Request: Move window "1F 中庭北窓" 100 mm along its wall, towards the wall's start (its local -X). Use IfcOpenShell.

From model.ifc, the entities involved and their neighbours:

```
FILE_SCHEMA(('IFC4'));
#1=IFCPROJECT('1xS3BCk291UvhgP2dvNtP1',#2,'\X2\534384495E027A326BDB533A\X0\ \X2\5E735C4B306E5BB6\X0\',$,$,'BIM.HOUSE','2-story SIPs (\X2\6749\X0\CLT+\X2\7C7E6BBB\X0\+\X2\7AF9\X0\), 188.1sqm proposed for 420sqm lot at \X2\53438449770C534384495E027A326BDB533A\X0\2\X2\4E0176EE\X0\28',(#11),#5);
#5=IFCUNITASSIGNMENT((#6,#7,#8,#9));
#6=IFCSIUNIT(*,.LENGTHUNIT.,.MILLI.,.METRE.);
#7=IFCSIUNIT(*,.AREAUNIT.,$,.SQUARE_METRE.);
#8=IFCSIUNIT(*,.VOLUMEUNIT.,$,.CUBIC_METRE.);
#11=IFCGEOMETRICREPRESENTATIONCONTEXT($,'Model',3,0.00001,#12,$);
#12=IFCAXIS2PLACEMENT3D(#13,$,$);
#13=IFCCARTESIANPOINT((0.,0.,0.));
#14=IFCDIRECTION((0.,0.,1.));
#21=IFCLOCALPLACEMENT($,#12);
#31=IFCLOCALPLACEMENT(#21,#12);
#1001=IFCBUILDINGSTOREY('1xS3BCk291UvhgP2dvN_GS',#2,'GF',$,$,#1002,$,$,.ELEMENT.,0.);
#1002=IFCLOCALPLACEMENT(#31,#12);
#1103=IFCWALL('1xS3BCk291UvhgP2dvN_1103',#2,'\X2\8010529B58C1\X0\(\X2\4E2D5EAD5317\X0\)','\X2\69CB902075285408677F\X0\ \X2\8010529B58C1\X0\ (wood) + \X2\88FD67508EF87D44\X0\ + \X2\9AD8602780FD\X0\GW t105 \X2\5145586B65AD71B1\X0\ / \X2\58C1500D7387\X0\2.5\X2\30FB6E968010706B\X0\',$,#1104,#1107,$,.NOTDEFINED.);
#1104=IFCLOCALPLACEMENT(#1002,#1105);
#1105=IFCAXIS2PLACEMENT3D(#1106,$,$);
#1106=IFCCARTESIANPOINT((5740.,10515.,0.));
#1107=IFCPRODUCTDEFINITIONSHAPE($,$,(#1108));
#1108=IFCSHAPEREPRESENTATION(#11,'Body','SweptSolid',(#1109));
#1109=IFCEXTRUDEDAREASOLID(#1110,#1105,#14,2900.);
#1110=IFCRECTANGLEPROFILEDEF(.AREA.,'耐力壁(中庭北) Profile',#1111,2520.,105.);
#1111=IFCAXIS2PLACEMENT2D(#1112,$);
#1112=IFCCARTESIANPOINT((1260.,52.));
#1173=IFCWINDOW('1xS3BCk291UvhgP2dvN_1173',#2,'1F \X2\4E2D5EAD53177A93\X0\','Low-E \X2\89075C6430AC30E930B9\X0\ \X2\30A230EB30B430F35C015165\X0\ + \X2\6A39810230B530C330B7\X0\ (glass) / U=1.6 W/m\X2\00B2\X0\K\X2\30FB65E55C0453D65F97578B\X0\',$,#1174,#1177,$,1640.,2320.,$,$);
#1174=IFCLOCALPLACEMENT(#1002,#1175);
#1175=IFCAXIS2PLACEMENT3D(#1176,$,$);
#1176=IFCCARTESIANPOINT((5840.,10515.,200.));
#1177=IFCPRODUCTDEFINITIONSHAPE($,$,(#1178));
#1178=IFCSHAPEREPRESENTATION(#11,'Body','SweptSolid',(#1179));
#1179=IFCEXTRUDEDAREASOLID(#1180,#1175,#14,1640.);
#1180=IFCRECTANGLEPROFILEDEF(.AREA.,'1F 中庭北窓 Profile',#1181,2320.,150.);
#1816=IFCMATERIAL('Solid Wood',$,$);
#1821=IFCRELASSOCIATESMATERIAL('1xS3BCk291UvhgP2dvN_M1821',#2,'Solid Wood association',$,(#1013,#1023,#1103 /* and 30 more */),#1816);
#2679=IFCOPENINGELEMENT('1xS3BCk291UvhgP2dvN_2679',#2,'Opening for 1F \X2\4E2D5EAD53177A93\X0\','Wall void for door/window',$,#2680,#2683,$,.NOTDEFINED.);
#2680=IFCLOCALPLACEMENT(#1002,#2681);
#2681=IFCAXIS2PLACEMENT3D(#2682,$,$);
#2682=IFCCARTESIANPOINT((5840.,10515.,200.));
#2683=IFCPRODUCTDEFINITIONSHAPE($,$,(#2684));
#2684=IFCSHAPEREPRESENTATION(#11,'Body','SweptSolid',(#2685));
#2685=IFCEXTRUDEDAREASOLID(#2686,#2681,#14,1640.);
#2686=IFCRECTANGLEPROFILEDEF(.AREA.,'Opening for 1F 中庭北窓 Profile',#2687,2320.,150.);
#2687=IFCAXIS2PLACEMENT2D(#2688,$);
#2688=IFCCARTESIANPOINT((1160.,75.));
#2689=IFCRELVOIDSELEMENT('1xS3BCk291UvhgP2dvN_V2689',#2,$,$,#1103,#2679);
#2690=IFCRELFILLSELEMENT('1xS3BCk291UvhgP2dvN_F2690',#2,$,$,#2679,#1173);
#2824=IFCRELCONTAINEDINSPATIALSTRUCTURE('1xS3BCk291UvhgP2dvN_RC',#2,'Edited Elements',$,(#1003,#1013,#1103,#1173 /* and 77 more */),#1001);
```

```python
import ifcopenshell
import ifcopenshell.api.geometry
import ifcopenshell.util.placement
import ifcopenshell.util.unit

model = ifcopenshell.open("model.ifc")
unit_scale = ifcopenshell.util.unit.calculate_unit_scale(model)

window = model.by_id(1173)
opening = window.FillsVoids[0].RelatingOpeningElement
wall = opening.VoidsElements[0].RelatingBuildingElement

wall_matrix = ifcopenshell.util.placement.get_local_placement(wall.ObjectPlacement)
shift = wall_matrix[:3, 0] * -0.1 / unit_scale
before = ifcopenshell.util.placement.get_local_placement(window.ObjectPlacement)[:3, 3].copy()

# The window is not placed relative to its opening, so move both.
for product in (opening, window):
    matrix = ifcopenshell.util.placement.get_local_placement(product.ObjectPlacement)
    matrix[:3, 3] += shift
    ifcopenshell.api.geometry.edit_object_placement(model, product=product, matrix=matrix, is_si=False)

after = ifcopenshell.util.placement.get_local_placement(window.ObjectPlacement)[:3, 3]
print("window moved by", (after - before).round(3) + 0.0)

model.write("model-out.ifc")
```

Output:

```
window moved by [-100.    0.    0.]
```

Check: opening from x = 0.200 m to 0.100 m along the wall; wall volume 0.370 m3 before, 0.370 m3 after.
